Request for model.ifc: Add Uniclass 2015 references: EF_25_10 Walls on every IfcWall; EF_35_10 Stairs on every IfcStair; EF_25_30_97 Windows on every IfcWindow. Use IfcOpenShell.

First a look at what the model holds.

```python
import ifcopenshell

model = ifcopenshell.open("model.ifc")
print(model.schema)
print("classifications:", [c.Name for c in model.by_type("IfcClassification")])
for ifc_class in ("IfcDoor", "IfcRoof", "IfcStair", "IfcWall", "IfcWindow"):
    print(ifc_class, len(model.by_type(ifc_class)))
```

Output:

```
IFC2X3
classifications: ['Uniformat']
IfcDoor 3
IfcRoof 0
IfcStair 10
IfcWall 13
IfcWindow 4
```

```python
import ifcopenshell
import ifcopenshell.api.classification

model = ifcopenshell.open("model.ifc")

# IFC2X3 requires Source and Edition and has no link from the project to the system.
system = model.create_entity("IfcClassification", Source="NBS", Edition="2015", Name="Uniclass 2015")

codes = {
    "IfcWall": ("EF_25_10", "Walls"),
    "IfcStair": ("EF_35_10", "Stairs"),
    "IfcWindow": ("EF_25_30_97", "Windows"),
}
for ifc_class, (code, name) in codes.items():
    products = model.by_type(ifc_class)
    ifcopenshell.api.classification.add_reference(
        model, products=products, classification=system, identification=code, name=name
    )
    print(code, len(products))

model.write("model_rev.ifc")
```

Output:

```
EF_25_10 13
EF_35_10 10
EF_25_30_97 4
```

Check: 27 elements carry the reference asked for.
